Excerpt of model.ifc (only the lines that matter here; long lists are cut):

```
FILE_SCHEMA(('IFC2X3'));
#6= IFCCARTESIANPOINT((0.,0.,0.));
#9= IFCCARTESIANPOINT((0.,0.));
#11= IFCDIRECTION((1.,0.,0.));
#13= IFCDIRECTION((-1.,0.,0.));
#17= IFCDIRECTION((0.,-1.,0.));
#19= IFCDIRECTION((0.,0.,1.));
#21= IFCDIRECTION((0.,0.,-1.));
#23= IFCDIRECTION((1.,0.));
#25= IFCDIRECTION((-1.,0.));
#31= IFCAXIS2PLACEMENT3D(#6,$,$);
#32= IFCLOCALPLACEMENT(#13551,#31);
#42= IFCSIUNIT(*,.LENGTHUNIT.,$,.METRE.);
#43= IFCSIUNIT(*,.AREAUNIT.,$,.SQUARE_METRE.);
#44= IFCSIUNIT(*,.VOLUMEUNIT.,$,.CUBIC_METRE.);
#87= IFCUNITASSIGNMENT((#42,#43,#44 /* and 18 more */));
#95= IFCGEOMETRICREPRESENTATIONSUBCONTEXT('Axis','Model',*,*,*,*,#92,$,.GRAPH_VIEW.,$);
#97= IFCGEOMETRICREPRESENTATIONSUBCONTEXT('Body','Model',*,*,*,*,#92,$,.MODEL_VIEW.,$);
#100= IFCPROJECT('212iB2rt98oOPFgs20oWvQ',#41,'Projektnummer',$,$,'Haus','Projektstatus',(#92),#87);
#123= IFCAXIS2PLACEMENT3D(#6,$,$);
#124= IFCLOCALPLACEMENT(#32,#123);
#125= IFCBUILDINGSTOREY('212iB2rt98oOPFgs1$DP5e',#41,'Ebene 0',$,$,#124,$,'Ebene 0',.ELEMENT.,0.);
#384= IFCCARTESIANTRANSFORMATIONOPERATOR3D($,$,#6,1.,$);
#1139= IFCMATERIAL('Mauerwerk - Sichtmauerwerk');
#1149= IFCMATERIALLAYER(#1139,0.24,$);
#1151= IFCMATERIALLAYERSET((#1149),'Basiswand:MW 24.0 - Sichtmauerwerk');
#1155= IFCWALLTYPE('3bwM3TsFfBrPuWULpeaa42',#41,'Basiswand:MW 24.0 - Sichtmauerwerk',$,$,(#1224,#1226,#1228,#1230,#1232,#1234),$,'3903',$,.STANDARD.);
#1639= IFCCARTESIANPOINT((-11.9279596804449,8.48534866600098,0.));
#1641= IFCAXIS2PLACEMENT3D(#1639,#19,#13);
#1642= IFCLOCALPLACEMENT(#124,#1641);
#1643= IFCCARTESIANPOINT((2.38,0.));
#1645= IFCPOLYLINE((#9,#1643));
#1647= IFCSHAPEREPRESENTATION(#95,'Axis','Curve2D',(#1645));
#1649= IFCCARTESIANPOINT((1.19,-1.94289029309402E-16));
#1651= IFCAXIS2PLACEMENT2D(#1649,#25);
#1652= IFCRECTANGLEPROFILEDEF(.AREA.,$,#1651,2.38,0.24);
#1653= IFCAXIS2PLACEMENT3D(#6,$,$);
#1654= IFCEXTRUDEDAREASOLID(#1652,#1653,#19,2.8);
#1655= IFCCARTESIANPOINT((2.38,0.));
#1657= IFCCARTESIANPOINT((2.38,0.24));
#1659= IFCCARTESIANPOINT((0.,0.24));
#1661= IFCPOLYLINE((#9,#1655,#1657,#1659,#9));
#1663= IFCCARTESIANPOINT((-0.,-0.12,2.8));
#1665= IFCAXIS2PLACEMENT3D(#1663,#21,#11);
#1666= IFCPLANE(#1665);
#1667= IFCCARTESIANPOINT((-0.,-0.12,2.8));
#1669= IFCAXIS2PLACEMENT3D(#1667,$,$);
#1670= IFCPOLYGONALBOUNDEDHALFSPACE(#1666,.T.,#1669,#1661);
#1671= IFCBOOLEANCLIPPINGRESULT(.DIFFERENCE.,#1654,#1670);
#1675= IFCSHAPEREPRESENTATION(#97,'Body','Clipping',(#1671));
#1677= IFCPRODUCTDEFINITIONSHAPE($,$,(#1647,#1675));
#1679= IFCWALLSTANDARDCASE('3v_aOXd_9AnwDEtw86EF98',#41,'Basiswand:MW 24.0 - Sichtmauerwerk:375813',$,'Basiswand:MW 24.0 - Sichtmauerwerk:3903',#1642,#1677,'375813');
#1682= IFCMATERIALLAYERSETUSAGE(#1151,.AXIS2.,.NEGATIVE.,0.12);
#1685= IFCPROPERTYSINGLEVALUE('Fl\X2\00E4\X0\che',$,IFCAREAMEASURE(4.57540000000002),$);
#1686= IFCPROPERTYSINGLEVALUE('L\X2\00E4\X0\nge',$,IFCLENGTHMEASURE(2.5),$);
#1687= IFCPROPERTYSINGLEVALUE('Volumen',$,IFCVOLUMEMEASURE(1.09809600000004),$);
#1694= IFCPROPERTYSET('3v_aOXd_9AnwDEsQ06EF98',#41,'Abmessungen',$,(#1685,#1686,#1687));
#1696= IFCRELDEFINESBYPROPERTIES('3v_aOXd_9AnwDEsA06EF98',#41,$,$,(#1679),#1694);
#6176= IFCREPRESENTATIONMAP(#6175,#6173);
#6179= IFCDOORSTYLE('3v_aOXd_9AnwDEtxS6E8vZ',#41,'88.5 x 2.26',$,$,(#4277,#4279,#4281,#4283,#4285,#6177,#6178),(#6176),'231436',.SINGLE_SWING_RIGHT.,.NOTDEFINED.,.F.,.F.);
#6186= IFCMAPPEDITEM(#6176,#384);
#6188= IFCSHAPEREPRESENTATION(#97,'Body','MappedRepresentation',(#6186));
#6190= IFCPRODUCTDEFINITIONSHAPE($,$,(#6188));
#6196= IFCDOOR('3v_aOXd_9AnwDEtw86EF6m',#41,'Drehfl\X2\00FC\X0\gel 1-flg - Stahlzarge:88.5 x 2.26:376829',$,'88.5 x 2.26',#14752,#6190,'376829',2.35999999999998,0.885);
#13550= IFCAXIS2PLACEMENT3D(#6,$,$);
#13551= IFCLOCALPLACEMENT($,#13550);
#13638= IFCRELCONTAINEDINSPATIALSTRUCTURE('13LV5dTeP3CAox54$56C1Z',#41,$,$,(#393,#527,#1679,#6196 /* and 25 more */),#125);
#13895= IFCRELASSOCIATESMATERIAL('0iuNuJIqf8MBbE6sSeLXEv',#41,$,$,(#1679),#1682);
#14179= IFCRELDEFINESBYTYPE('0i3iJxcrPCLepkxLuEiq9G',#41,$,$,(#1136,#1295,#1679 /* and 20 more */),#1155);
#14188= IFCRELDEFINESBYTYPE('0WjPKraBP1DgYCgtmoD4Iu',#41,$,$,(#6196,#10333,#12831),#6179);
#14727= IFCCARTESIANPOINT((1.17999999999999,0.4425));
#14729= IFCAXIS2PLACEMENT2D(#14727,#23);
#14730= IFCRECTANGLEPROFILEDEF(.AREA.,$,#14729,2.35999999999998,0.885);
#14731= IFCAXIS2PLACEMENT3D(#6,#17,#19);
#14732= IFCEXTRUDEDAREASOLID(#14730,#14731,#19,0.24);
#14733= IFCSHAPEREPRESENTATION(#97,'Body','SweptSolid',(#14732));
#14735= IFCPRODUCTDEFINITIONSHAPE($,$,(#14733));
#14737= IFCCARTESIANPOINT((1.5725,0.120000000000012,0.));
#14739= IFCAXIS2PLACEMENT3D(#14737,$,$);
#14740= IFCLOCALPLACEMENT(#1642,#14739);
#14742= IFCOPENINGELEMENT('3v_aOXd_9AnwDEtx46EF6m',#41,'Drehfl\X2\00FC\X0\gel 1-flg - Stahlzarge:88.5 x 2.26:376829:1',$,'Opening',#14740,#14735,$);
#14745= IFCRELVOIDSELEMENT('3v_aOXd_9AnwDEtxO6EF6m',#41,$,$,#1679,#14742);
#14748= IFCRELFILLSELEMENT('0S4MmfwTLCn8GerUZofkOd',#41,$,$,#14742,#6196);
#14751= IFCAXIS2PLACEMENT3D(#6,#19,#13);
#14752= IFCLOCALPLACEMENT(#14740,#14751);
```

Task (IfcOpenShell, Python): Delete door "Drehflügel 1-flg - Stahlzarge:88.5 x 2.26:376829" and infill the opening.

```python
import ifcopenshell
import ifcopenshell.api.feature
import ifcopenshell.api.pset
import ifcopenshell.api.root
import ifcopenshell.geom
import ifcopenshell.util.element
import ifcopenshell.util.shape
import ifcopenshell.util.unit

model = ifcopenshell.open("model.ifc")
area_scale = ifcopenshell.util.unit.calculate_unit_scale(model, "AREAUNIT")
volume_scale = ifcopenshell.util.unit.calculate_unit_scale(model, "VOLUMEUNIT")
settings = ifcopenshell.geom.settings()


def volume(element):
    """Net volume in cubic metres, openings subtracted."""
    shape = ifcopenshell.geom.create_shape(settings, element)
    return ifcopenshell.util.shape.get_volume(shape.geometry)


door = model.by_guid("3v_aOXd_9AnwDEtw86EF6m")
opening = door.FillsVoids[0].RelatingOpeningElement
wall = opening.VoidsElements[0].RelatingBuildingElement
before = volume(wall)

ifcopenshell.api.root.remove_product(model, product=door)
ifcopenshell.api.feature.remove_feature(model, feature=opening)

after = volume(wall)
thickness = 0.24  # wall thickness in metres

# Update the wall's stored quantities.
pset = model.by_id(ifcopenshell.util.element.get_pset(wall, "Abmessungen", should_inherit=False)["id"])
ifcopenshell.api.pset.edit_pset(model, pset=pset, properties={
    "Fläche": model.create_entity("IfcAreaMeasure", after / thickness / area_scale),
    "Volumen": model.create_entity("IfcVolumeMeasure", after / volume_scale),
})

print(f"wall volume {before:.3f} -> {after:.3f} m3")

model.write("model_rev.ifc")
```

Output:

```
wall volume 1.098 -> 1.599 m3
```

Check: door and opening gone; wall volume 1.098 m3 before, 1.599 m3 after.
